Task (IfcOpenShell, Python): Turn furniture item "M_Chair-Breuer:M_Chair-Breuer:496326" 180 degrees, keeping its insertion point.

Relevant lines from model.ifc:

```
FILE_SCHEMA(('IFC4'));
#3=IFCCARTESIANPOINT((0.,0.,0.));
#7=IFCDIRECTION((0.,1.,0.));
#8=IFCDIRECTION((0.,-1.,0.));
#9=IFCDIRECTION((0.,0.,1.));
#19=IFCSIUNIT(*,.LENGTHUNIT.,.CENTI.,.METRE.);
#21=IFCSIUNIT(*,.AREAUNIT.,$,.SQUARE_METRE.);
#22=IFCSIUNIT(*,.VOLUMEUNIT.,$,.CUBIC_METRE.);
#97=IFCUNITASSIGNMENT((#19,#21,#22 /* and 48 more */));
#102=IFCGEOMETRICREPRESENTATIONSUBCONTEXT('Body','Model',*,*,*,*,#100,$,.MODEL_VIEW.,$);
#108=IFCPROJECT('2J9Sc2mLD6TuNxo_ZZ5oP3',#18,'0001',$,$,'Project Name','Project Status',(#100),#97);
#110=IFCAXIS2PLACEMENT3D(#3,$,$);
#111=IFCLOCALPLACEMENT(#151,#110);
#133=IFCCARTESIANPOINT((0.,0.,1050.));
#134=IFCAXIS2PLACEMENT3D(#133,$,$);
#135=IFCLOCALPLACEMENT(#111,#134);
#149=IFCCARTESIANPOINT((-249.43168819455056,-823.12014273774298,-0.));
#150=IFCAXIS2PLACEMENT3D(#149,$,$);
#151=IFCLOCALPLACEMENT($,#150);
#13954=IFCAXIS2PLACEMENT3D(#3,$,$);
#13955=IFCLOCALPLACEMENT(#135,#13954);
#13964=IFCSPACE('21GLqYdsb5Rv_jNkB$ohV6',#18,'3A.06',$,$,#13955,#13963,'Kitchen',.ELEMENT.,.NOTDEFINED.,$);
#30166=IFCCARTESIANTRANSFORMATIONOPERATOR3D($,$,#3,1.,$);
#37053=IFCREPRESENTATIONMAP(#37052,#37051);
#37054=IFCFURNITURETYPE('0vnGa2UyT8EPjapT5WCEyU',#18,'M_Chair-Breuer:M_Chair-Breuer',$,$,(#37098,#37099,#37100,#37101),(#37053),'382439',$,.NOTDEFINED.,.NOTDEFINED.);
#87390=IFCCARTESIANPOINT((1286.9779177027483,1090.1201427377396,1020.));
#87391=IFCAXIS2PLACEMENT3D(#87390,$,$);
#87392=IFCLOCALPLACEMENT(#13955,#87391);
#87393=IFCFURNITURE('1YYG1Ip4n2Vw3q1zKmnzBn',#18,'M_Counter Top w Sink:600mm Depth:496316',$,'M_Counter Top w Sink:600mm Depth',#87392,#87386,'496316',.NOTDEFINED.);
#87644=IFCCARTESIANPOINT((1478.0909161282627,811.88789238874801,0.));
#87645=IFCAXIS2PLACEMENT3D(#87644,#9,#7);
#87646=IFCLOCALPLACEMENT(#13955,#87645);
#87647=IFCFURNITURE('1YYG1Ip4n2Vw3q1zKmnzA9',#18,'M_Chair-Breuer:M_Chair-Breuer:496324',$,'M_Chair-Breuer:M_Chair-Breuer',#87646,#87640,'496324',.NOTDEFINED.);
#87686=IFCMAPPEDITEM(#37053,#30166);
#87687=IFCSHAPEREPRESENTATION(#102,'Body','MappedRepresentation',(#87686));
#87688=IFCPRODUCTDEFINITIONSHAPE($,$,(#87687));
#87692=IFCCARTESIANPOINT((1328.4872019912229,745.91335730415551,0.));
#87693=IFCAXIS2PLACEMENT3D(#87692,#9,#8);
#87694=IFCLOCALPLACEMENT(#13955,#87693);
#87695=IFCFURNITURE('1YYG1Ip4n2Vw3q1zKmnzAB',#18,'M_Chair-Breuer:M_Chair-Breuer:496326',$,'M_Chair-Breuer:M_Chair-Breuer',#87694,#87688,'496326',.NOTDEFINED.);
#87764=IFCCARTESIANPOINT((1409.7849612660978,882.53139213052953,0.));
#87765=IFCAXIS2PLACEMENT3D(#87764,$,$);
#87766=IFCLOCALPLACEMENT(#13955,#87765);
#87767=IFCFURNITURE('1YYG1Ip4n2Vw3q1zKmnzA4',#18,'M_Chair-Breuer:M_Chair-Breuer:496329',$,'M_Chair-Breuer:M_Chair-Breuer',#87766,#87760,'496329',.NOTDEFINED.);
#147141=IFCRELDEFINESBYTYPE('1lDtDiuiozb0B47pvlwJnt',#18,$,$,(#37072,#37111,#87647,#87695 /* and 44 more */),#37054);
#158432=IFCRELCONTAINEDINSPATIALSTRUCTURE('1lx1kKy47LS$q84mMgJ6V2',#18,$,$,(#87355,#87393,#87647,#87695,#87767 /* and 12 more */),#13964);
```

```python
import ifcopenshell
import ifcopenshell.api.geometry
import ifcopenshell.util.placement

model = ifcopenshell.open("model.ifc")

item = model.by_guid("1YYG1Ip4n2Vw3q1zKmnzAB")
matrix = ifcopenshell.util.placement.get_local_placement(item.ObjectPlacement)
matrix = matrix @ ifcopenshell.util.placement.rotation(180, "Z")
ifcopenshell.api.geometry.edit_object_placement(model, product=item, matrix=matrix, is_si=False)

print(ifcopenshell.util.placement.get_local_placement(item.ObjectPlacement).round(3) + 0.0)

model.write("model-out.ifc")
```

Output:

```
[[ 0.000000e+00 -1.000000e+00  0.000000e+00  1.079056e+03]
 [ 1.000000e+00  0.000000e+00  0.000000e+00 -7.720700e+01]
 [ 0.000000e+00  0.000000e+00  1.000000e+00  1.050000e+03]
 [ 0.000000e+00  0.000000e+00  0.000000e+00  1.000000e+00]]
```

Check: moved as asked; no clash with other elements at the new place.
